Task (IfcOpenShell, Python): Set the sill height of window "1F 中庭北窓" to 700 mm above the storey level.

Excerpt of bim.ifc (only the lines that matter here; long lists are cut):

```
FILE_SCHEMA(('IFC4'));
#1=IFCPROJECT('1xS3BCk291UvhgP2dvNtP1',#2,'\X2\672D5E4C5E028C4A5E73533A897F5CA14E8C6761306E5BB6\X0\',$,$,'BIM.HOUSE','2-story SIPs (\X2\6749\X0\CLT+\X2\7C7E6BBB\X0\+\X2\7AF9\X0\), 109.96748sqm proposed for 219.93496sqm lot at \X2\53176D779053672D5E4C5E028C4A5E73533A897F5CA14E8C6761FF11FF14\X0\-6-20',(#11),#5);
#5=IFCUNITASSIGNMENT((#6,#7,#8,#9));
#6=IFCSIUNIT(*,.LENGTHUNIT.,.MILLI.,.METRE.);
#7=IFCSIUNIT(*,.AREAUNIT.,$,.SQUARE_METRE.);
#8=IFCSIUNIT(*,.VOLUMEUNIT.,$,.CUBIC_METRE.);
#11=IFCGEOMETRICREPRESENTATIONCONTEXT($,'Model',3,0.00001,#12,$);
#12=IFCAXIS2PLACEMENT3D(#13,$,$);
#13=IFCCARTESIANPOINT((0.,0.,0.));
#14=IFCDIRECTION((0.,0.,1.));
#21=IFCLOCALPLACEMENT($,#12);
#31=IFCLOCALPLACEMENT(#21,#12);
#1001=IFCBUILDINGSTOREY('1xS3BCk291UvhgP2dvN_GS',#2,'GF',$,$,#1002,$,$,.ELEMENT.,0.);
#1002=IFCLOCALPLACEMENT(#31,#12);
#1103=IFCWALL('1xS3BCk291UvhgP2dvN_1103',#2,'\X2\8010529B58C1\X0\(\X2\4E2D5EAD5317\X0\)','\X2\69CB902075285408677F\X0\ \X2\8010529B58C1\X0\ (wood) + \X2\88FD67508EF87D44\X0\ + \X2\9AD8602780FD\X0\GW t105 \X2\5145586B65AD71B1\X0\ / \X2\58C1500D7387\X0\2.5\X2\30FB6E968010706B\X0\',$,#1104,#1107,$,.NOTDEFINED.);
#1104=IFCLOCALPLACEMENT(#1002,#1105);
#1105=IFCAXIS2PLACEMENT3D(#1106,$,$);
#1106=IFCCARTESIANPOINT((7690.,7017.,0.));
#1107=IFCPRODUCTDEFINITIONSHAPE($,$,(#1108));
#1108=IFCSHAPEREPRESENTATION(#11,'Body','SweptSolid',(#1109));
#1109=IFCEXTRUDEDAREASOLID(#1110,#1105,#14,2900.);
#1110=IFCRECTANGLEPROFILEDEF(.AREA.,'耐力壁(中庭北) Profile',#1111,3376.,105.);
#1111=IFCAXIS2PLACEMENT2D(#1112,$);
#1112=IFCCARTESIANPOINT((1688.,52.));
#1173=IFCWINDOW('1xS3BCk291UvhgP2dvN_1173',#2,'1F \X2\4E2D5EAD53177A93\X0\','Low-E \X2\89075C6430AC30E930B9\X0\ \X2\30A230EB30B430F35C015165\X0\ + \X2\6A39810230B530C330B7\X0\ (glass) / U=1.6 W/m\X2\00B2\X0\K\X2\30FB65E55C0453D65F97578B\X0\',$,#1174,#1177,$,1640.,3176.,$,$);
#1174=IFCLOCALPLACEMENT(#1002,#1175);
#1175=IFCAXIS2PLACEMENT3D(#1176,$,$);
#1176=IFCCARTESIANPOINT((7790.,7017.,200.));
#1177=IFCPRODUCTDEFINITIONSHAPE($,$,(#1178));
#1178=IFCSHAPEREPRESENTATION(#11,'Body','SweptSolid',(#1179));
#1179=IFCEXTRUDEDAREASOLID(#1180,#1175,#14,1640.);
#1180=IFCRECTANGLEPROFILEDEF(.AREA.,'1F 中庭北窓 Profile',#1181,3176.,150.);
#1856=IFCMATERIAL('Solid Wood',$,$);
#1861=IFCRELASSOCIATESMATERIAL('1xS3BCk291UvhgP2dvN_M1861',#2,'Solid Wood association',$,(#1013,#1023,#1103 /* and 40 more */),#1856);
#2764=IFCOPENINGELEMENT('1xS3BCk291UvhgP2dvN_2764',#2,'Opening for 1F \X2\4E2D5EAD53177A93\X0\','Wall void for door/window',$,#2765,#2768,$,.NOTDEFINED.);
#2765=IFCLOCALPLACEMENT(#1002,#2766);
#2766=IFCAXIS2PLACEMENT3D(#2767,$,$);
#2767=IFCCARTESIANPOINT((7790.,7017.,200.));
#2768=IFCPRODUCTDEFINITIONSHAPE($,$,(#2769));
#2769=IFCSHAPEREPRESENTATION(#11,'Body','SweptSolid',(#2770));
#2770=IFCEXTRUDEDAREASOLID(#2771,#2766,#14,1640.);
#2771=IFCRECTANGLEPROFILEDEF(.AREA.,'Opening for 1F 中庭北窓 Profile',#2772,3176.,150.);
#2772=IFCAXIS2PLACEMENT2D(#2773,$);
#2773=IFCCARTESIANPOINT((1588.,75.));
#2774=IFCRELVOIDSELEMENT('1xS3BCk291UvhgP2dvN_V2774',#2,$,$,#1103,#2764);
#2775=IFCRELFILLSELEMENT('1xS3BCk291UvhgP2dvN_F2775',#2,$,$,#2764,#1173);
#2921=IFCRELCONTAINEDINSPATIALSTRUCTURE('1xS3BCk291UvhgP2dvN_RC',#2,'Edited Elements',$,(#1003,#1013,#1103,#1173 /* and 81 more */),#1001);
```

```python
import numpy as np
import ifcopenshell
import ifcopenshell.api.geometry
import ifcopenshell.geom
import ifcopenshell.util.element
import ifcopenshell.util.placement
import ifcopenshell.util.shape
import ifcopenshell.util.unit

model = ifcopenshell.open("bim.ifc")
unit_scale = ifcopenshell.util.unit.calculate_unit_scale(model)

window = model.by_id(1173)
opening = window.FillsVoids[0].RelatingOpeningElement
storey = ifcopenshell.util.element.get_container(window, ifc_class="IfcBuildingStorey")
level = ifcopenshell.util.placement.get_local_placement(storey.ObjectPlacement)[2, 3]

# The opening's origin need not be at the sill, so measure its lowest point.
shape = ifcopenshell.geom.create_shape(ifcopenshell.geom.settings(), opening)
bottom = ifcopenshell.util.shape.get_shape_bottom_elevation(shape, shape.geometry) / unit_scale
dz = level + 0.7 / unit_scale - bottom

shift = np.array([0.0, 0.0, dz])
# The window is not placed relative to its opening, so move both.
for product in (opening, window):
    matrix = ifcopenshell.util.placement.get_local_placement(product.ObjectPlacement)
    matrix[:3, 3] += shift
    ifcopenshell.api.geometry.edit_object_placement(model, product=product, matrix=matrix, is_si=False)

print(f"moved by {dz * unit_scale:+.3f} m")

model.write("bim_updated.ifc")
```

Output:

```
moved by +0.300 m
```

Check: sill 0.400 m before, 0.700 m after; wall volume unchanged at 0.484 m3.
